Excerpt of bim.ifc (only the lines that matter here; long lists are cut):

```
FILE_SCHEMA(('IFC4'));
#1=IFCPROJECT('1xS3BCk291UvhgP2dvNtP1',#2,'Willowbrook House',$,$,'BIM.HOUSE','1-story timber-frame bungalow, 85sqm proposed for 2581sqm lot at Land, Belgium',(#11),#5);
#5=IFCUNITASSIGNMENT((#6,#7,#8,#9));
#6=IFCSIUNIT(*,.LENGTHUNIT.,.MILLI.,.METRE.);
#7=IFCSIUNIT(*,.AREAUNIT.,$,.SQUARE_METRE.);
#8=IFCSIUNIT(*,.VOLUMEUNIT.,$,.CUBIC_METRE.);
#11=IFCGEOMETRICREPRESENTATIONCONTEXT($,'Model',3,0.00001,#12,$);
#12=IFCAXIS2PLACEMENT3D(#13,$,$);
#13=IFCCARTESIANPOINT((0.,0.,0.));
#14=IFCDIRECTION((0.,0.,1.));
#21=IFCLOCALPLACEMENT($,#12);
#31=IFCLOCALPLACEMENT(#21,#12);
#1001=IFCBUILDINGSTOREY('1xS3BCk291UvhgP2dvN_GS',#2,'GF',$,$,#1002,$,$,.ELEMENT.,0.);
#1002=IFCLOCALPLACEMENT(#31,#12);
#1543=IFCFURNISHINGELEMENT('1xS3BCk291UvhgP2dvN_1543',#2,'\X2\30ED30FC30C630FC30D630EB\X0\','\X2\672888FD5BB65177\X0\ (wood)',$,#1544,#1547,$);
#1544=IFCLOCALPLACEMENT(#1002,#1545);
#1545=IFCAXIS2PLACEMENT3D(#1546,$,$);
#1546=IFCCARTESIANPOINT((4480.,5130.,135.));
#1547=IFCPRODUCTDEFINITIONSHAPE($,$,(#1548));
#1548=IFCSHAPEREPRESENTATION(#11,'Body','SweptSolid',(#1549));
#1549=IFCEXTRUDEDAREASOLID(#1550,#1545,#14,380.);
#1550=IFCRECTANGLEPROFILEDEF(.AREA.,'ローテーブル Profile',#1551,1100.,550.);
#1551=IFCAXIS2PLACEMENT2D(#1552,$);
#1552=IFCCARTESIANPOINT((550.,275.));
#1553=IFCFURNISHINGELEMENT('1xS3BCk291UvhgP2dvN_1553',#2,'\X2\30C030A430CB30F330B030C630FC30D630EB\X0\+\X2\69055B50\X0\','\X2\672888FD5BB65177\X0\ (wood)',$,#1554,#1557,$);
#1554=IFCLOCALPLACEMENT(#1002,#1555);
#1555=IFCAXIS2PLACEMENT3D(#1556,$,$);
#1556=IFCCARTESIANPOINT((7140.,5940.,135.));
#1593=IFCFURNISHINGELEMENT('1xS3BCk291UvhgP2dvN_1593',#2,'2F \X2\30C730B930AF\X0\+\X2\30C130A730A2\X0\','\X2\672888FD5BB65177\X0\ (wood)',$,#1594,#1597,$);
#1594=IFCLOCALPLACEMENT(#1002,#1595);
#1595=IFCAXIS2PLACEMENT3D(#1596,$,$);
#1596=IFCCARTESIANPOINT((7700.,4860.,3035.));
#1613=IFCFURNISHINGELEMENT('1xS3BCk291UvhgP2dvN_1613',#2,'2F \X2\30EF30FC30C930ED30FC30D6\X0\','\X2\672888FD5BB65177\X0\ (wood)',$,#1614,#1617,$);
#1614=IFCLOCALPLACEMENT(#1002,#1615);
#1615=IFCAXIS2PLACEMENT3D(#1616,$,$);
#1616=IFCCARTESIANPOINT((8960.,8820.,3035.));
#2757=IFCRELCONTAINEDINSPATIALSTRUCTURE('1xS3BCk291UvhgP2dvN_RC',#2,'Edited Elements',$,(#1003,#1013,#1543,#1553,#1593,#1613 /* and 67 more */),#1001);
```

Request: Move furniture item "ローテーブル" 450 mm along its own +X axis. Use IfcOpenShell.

```python
import ifcopenshell
import ifcopenshell.api.geometry
import ifcopenshell.util.placement

model = ifcopenshell.open("bim.ifc")

item = model.by_guid("1xS3BCk291UvhgP2dvN_1543")
matrix = ifcopenshell.util.placement.get_local_placement(item.ObjectPlacement)
matrix[:3, 3] += matrix[:3, 0] * 450.0
ifcopenshell.api.geometry.edit_object_placement(model, product=item, matrix=matrix, is_si=False)

print(ifcopenshell.util.placement.get_local_placement(item.ObjectPlacement).round(3) + 0.0)

model.write("bim_rev.ifc")
```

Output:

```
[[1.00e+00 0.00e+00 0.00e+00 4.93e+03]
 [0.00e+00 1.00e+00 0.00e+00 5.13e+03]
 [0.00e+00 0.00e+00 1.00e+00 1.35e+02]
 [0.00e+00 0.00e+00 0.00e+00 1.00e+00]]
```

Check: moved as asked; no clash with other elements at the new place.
